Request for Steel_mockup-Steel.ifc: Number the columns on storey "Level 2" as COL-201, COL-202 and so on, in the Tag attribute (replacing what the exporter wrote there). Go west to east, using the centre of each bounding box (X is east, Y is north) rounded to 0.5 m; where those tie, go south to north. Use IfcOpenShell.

First a look at what the model holds.

```python
import ifcopenshell
import ifcopenshell.util.element
import ifcopenshell.util.placement

model = ifcopenshell.open("Steel_mockup-Steel.ifc")
print(model.schema)
storey = next(s for s in model.by_type("IfcBuildingStorey") if s.Name == "Level 2")
columns = [e for e in ifcopenshell.util.element.get_decomposition(storey) if e.is_a("IfcColumn")]
for e in sorted(columns, key=lambda e: e.id()):
    origin = ifcopenshell.util.placement.get_local_placement(e.ObjectPlacement)[:3, 3]
    print(e.id(), e.Tag, e.Name, origin.round(2) + 0.0, sep=" | ")
```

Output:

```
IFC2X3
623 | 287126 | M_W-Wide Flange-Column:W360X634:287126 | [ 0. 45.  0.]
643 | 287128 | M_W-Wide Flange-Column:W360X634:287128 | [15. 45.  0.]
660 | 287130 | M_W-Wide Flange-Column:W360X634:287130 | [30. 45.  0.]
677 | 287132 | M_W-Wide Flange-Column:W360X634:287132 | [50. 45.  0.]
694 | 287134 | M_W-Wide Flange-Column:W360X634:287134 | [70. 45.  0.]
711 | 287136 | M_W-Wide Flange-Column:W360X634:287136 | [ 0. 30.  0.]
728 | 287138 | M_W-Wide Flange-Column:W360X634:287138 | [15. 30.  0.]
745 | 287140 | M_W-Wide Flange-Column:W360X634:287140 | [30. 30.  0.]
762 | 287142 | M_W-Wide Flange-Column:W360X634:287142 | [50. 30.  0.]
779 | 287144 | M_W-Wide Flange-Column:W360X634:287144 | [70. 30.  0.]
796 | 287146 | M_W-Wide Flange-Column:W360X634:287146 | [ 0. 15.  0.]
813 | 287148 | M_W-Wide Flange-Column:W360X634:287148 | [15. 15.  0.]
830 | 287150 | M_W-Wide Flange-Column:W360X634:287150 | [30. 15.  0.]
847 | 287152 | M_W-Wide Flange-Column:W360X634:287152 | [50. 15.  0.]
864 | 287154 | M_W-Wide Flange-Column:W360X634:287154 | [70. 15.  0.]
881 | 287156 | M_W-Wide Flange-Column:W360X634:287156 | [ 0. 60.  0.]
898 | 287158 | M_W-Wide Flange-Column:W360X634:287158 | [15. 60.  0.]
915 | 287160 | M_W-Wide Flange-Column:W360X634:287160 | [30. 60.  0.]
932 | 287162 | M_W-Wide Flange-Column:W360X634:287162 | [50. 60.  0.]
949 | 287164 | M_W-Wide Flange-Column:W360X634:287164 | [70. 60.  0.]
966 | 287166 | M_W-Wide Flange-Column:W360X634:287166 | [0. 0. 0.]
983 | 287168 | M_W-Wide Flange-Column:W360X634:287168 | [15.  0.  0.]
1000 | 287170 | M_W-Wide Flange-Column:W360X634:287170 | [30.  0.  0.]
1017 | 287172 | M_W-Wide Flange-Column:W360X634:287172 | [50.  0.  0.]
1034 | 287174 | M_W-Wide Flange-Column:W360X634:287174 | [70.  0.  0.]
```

```python
import ifcopenshell
import ifcopenshell.geom
import ifcopenshell.util.element
import ifcopenshell.util.shape

model = ifcopenshell.open("Steel_mockup-Steel.ifc")
settings = ifcopenshell.geom.settings()
settings.set("use-world-coords", True)


def centre(element):
    shape = ifcopenshell.geom.create_shape(settings, element)
    return ifcopenshell.util.shape.get_bbox_centroid(shape.geometry)


storey = next(s for s in model.by_type("IfcBuildingStorey") if s.Name == "Level 2")
columns = [e for e in ifcopenshell.util.element.get_decomposition(storey) if e.is_a("IfcColumn")]

# Insertion points can sit at a corner or the storey origin, so sort by the geometry (in metres).
centres = {e: centre(e) for e in columns}
columns.sort(key=lambda e: (round(centres[e][0] / 0.5), centres[e][1]))

for i, e in enumerate(columns, start=1):
    number = f"COL-2{i:02d}"
    e.Tag = number
    print(e.id(), number)

model.write("Steel_mockup-Steel_rev.ifc")
```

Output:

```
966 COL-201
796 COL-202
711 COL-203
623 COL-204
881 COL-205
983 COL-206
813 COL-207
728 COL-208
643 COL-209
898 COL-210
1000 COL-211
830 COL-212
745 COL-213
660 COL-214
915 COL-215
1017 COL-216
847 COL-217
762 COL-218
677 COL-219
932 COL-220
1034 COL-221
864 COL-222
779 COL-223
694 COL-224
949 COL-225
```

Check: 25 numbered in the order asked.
